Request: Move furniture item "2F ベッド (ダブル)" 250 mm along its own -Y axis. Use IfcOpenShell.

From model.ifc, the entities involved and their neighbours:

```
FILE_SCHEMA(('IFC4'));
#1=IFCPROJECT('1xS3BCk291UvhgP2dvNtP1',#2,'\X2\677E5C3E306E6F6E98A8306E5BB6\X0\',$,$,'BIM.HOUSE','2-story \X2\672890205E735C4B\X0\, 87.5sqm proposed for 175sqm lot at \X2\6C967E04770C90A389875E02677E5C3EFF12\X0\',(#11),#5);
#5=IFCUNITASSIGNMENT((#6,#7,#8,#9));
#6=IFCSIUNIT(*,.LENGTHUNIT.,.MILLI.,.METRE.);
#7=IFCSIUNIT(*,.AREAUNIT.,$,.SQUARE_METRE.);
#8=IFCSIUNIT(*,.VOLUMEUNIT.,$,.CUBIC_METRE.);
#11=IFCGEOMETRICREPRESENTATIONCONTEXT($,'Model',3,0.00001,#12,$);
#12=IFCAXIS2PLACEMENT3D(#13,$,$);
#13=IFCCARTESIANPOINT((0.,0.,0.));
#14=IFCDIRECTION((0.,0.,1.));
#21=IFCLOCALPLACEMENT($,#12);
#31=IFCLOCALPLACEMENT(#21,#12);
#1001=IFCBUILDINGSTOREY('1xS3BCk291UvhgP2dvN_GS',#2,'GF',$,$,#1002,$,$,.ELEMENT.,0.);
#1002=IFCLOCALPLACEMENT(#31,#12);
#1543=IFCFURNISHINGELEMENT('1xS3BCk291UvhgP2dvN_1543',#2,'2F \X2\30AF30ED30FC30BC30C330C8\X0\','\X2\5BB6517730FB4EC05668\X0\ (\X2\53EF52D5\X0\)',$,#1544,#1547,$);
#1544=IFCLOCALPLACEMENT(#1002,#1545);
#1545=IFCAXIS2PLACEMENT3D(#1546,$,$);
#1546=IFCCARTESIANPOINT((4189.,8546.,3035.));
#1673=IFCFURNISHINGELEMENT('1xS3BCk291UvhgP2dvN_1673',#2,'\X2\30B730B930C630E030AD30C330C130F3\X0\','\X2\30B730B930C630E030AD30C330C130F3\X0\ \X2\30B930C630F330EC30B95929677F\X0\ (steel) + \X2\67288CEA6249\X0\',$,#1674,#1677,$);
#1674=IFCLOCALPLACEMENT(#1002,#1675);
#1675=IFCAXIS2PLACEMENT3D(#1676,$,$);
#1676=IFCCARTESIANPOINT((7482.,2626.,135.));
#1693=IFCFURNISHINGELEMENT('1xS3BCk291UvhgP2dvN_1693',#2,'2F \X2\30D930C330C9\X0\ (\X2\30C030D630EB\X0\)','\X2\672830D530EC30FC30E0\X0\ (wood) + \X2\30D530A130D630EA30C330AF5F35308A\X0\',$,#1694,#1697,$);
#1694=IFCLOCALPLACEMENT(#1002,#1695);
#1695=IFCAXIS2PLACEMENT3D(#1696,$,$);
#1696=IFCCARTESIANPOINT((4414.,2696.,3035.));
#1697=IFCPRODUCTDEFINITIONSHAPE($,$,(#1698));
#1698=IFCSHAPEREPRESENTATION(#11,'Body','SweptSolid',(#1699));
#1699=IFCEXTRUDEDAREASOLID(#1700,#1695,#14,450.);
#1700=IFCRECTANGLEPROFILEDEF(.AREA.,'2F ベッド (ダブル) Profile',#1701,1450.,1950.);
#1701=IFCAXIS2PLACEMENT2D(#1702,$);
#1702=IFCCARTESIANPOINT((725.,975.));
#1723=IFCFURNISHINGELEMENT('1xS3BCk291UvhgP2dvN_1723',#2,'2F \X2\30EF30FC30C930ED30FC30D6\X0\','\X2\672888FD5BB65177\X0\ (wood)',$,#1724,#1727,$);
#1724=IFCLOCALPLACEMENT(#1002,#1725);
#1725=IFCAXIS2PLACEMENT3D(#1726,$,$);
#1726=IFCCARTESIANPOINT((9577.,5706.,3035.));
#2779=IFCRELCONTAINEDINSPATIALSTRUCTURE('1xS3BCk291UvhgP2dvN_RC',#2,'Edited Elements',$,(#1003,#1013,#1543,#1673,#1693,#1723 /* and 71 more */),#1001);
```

```python
import ifcopenshell
import ifcopenshell.api.geometry
import ifcopenshell.util.placement
import ifcopenshell.util.unit

model = ifcopenshell.open("model.ifc")
unit_scale = ifcopenshell.util.unit.calculate_unit_scale(model)

item = model.by_guid("1xS3BCk291UvhgP2dvN_1693")
matrix = ifcopenshell.util.placement.get_local_placement(item.ObjectPlacement)
matrix[:3, 3] -= matrix[:3, 1] * 0.25 / unit_scale
ifcopenshell.api.geometry.edit_object_placement(model, product=item, matrix=matrix, is_si=False)

print(ifcopenshell.util.placement.get_local_placement(item.ObjectPlacement).round(3) + 0.0)

model.write("model_edited.ifc")
```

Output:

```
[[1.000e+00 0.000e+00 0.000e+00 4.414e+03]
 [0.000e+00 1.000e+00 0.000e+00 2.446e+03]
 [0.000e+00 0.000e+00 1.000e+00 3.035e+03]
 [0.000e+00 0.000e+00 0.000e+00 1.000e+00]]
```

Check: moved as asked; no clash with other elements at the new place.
